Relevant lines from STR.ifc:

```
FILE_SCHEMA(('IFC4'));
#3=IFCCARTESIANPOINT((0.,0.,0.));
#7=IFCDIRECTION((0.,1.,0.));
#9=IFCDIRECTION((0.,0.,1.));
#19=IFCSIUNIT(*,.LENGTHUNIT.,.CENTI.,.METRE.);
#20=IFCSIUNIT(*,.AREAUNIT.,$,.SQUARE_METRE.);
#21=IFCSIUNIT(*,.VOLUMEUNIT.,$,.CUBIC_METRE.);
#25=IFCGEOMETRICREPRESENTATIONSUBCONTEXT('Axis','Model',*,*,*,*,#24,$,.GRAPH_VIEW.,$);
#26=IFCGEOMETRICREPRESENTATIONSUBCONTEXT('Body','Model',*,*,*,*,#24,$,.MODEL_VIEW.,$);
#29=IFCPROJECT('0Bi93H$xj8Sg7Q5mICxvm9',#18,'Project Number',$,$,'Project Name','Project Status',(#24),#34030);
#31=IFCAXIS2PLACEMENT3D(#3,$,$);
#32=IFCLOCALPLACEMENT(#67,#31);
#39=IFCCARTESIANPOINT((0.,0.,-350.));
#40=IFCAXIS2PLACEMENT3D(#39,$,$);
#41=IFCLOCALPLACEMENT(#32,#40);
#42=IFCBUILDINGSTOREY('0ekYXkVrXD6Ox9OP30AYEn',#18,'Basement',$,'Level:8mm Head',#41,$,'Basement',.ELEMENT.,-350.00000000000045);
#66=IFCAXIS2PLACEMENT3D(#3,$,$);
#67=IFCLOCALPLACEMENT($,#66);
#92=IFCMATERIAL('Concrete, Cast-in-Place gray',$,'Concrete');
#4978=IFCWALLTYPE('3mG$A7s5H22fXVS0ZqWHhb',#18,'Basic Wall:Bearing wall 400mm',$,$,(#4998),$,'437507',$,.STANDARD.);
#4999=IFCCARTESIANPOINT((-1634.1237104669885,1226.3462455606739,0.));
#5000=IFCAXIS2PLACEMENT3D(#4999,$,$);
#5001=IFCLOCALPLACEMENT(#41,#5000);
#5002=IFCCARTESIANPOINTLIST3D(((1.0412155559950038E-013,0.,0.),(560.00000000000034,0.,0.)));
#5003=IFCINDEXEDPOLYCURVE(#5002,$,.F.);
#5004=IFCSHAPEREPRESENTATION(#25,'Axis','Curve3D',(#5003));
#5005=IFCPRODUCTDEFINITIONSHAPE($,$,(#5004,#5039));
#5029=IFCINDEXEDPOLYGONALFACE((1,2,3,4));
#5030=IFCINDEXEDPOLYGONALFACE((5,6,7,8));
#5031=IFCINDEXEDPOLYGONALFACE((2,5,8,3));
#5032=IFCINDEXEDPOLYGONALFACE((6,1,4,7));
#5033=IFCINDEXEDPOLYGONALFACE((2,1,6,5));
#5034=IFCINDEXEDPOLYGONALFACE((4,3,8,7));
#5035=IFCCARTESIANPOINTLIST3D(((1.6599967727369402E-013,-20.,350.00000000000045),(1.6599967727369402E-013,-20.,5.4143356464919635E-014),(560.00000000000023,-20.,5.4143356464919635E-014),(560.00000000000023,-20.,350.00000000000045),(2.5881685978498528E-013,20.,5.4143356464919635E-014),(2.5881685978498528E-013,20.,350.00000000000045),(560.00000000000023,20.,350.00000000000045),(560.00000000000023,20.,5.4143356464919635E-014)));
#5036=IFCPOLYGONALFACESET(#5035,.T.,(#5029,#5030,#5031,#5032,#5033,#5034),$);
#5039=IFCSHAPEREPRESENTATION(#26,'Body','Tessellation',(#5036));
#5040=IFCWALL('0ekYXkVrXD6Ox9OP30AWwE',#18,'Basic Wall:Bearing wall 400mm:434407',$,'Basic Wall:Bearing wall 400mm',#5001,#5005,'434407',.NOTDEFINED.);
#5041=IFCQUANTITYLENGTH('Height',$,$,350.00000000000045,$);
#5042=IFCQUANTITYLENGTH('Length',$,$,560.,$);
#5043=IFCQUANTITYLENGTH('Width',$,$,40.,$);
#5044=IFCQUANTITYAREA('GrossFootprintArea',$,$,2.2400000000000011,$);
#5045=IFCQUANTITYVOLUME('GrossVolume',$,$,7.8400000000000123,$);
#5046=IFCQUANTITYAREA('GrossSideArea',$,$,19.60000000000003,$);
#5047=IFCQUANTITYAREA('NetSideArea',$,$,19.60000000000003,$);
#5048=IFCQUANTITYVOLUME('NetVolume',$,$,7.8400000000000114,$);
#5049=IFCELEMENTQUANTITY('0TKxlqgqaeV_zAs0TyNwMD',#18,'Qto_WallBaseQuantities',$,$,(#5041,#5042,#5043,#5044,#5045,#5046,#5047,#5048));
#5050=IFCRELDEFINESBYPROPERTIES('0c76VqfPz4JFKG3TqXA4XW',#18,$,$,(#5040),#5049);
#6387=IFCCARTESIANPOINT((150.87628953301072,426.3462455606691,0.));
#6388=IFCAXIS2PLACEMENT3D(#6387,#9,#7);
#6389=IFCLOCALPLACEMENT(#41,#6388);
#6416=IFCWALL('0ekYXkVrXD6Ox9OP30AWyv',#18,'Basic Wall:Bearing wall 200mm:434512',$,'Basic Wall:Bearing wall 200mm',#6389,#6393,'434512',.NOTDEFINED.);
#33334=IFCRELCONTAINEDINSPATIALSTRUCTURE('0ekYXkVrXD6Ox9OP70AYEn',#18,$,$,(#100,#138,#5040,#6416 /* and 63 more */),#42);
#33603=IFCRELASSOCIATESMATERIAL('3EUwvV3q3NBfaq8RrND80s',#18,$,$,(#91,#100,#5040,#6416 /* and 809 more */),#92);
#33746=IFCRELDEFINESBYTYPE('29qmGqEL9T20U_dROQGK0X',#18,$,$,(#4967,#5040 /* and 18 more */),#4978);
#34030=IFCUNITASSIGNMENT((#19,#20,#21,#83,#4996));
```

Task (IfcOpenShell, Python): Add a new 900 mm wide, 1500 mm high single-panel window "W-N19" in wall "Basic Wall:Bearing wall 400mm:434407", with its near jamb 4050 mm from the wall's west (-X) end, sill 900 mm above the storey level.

```python
import numpy as np
import ifcopenshell
import ifcopenshell.api.feature
import ifcopenshell.api.geometry
import ifcopenshell.api.pset
import ifcopenshell.api.root
import ifcopenshell.api.spatial
import ifcopenshell.geom
import ifcopenshell.util.element
import ifcopenshell.util.placement
import ifcopenshell.util.representation
import ifcopenshell.util.shape
import ifcopenshell.util.unit

model = ifcopenshell.open("STR.ifc")
unit_scale = ifcopenshell.util.unit.calculate_unit_scale(model)
area_scale = ifcopenshell.util.unit.calculate_unit_scale(model, "AREAUNIT")
volume_scale = ifcopenshell.util.unit.calculate_unit_scale(model, "VOLUMEUNIT")
settings = ifcopenshell.geom.settings()


def volume(element):
    """Net volume in cubic metres, openings subtracted."""
    shape = ifcopenshell.geom.create_shape(settings, element)
    return ifcopenshell.util.shape.get_volume(shape.geometry)


wall = model.by_guid("0ekYXkVrXD6Ox9OP30AWwE")
storey = ifcopenshell.util.element.get_container(wall, ifc_class="IfcBuildingStorey")
context = ifcopenshell.util.representation.get_context(model, "Model", "Body", "MODEL_VIEW")
before = volume(wall)

width, height, from_end, sill = 0.9, 1.5, 4.05, 0.9  # metres

# The wall runs along its own X axis, and the end named is its -X end.
wall_shape = ifcopenshell.geom.create_shape(settings, wall)
x, y, z = ifcopenshell.util.shape.get_vertices(wall_shape.geometry).T
start = x.min() + from_end
face, thickness = float(y.min()), float(y.max() - y.min())
wall_matrix = ifcopenshell.util.placement.get_local_placement(wall.ObjectPlacement)
level = ifcopenshell.util.placement.get_local_placement(storey.ObjectPlacement)[2, 3]


def in_wall(x, y):
    """Placement at x, y metres in the wall's axes, at sill height."""
    matrix = wall_matrix.copy()
    matrix[:, 3] = wall_matrix @ np.array([x / unit_scale, y / unit_scale, 0.0, 1.0])
    matrix[2, 3] = level + sill / unit_scale
    return matrix


# Opening: a box that overshoots both wall faces by 50 mm.
opening = ifcopenshell.api.root.create_entity(model, ifc_class="IfcOpeningElement", predefined_type="OPENING")
box = ifcopenshell.api.geometry.add_wall_representation(
    model, context=context, length=width, height=height, thickness=thickness + 0.1
)
ifcopenshell.api.geometry.assign_representation(model, product=opening, representation=box)
ifcopenshell.api.geometry.edit_object_placement(model, product=opening, matrix=in_wall(start, face - 0.05), is_si=False)
ifcopenshell.api.feature.add_feature(model, feature=opening, element=wall)

window = ifcopenshell.api.root.create_entity(model, ifc_class="IfcWindow", name="W-N19", predefined_type="WINDOW")
window.OverallWidth, window.OverallHeight = width / unit_scale, height / unit_scale
window.PartitioningType = "SINGLE_PANEL"
body = ifcopenshell.api.geometry.add_window_representation(
    model,
    context=context,
    overall_width=window.OverallWidth,
    overall_height=window.OverallHeight,
    partition_type="SINGLE_PANEL",
)
ifcopenshell.api.geometry.assign_representation(model, product=window, representation=body)
ifcopenshell.api.spatial.assign_container(model, products=[window], relating_structure=storey)
ifcopenshell.api.feature.add_filling(model, opening=opening, element=window)

# Centre the window in the wall's thickness.
ifcopenshell.api.geometry.edit_object_placement(model, product=window, matrix=in_wall(start, face), is_si=False)
window_shape = ifcopenshell.geom.create_shape(settings, window)
depth = ifcopenshell.util.shape.get_vertices(window_shape.geometry)[:, 1]
offset = face + thickness / 2 - (depth.min() + depth.max()) / 2
ifcopenshell.api.geometry.edit_object_placement(model, product=window, matrix=in_wall(start, offset), is_si=False)

after = volume(wall)

# Update the wall's stored quantities.
qto = model.by_id(ifcopenshell.util.element.get_pset(wall, "Qto_WallBaseQuantities", should_inherit=False)["id"])
ifcopenshell.api.pset.edit_qto(model, qto=qto, properties={
    "NetSideArea": after / thickness / area_scale,
    "NetVolume": after / volume_scale,
})

print(f"wall volume {before:.3f} -> {after:.3f} m3")

model.write("STR_edited.ifc")
```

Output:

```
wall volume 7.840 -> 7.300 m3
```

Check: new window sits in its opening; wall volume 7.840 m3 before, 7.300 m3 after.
